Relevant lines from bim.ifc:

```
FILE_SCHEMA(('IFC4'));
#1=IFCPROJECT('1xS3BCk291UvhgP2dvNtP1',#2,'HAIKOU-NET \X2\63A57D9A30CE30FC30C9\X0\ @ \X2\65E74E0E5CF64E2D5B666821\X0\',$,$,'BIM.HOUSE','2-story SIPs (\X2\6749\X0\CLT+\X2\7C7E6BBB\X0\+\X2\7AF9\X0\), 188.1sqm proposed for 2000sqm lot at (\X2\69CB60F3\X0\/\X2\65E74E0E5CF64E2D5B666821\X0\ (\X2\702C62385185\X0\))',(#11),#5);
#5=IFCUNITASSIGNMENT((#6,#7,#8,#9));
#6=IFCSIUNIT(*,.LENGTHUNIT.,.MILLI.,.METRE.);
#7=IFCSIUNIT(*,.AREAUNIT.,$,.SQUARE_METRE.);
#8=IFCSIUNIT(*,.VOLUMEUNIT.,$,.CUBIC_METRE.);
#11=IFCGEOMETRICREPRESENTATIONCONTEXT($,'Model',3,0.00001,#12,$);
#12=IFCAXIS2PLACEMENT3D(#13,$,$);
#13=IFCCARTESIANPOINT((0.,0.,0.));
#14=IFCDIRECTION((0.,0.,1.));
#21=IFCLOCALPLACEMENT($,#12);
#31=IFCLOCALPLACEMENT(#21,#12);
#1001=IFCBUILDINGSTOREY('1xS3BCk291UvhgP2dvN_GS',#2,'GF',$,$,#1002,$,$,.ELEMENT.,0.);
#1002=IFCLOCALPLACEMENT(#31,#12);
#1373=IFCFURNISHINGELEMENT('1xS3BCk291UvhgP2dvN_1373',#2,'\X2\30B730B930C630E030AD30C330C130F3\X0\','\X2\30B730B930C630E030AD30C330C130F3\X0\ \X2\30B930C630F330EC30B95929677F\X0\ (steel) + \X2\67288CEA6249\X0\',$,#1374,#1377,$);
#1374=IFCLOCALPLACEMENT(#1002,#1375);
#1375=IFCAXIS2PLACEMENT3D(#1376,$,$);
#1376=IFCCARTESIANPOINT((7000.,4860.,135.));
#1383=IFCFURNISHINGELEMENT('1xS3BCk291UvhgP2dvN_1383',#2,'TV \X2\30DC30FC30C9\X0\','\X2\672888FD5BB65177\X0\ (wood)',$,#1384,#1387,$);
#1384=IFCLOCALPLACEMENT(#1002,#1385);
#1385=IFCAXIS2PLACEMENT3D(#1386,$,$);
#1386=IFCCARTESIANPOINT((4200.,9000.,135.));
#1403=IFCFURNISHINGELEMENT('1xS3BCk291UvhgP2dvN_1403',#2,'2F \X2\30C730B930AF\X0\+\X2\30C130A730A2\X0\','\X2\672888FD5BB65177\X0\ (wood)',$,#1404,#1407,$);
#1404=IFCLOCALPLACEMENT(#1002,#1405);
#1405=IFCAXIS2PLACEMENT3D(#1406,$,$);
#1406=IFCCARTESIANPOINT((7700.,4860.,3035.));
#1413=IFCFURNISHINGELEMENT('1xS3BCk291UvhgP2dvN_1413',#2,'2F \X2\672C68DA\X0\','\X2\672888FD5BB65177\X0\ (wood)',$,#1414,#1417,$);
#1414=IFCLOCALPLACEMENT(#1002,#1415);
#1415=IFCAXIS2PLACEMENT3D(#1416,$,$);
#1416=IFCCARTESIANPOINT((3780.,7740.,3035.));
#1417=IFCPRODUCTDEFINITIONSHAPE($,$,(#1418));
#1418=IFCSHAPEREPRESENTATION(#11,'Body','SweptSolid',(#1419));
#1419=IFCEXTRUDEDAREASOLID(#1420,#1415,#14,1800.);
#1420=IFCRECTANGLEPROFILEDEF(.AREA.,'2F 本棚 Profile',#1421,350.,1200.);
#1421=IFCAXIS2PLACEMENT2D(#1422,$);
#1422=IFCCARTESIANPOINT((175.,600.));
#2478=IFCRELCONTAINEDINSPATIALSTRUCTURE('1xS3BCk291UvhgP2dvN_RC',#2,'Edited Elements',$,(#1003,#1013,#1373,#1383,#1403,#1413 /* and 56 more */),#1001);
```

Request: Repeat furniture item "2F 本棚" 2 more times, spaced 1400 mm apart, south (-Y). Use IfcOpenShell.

```python
import numpy as np
import ifcopenshell
import ifcopenshell.api.geometry
import ifcopenshell.api.root
import ifcopenshell.util.element
import ifcopenshell.util.placement
import ifcopenshell.util.unit

model = ifcopenshell.open("bim.ifc")
unit_scale = ifcopenshell.util.unit.calculate_unit_scale(model)


def reuse_history(source, copy):
    """copy_class also copies each property set's owner history, people and application; keep the originals."""
    for rel in copy.IsDefinedBy:
        if rel.is_a("IfcRelDefinesByProperties") and (history := rel.RelatingPropertyDefinition.OwnerHistory):
            rel.RelatingPropertyDefinition.OwnerHistory = source.OwnerHistory
            ifcopenshell.util.element.remove_deep2(model, history)


source = model.by_guid("1xS3BCk291UvhgP2dvN_1413")
base = ifcopenshell.util.placement.get_local_placement(source.ObjectPlacement)
step = np.array([0.0, -1.0, 0.0]) * 1.4 / unit_scale

for i in range(1, 3):
    copy = ifcopenshell.api.root.copy_class(model, product=source)
    copy.Representation = ifcopenshell.util.element.copy_deep(
        model, source.Representation, exclude=["IfcGeometricRepresentationContext", "IfcRepresentationMap"]
    )
    reuse_history(source, copy)
    matrix = base.copy()
    matrix[:3, 3] += i * step
    print("added at", matrix[:3, 3].round(3) + 0.0)
    ifcopenshell.api.geometry.edit_object_placement(model, product=copy, matrix=matrix, is_si=False)

model.write("bim_edited.ifc")
```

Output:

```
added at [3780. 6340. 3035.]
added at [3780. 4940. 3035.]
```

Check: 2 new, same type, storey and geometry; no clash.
